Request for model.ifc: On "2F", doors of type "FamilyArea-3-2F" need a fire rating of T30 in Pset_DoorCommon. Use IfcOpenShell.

First a look at what the model holds.

```python
import ifcopenshell
import ifcopenshell.util.element

model = ifcopenshell.open("model.ifc")
print(model.schema)
storey = next(s for s in model.by_type("IfcBuildingStorey") if s.Name == "2F")
doors = [e for e in ifcopenshell.util.element.get_decomposition(storey) if e.is_a("IfcDoor")]
seen = {}
for e in doors:
    element_type = ifcopenshell.util.element.get_type(e)
    key = (element_type.Name if element_type != e and element_type else None, ifcopenshell.util.element.get_pset(e, "Pset_DoorCommon", "FireRating"))
    seen[key] = seen.get(key, 0) + 1
for (name, value), count in sorted(seen.items(), key=str):
    print(count, "x", name, "|", value)
```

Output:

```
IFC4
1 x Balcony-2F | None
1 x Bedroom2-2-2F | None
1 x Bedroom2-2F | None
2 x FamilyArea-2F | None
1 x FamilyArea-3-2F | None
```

```python
import ifcopenshell
import ifcopenshell.api.pset
import ifcopenshell.util.element

model = ifcopenshell.open("model.ifc")

storey = next(s for s in model.by_type("IfcBuildingStorey") if s.Name == "2F")
doors = [e for e in ifcopenshell.util.element.get_decomposition(storey) if e.is_a("IfcDoor")]

count = 0
for e in doors:
    element_type = ifcopenshell.util.element.get_type(e)
    if element_type in (None, e) or element_type.Name != "FamilyArea-3-2F":
        continue
    # add_pset returns the element's existing set when there is one.
    pset = ifcopenshell.api.pset.add_pset(model, product=e, name="Pset_DoorCommon")
    ifcopenshell.api.pset.edit_pset(model, pset=pset, properties={"FireRating": "T30"})
    count += 1

print(count, "doors updated")

model.write("model_edited.ifc")
```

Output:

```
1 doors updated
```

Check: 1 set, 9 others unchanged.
